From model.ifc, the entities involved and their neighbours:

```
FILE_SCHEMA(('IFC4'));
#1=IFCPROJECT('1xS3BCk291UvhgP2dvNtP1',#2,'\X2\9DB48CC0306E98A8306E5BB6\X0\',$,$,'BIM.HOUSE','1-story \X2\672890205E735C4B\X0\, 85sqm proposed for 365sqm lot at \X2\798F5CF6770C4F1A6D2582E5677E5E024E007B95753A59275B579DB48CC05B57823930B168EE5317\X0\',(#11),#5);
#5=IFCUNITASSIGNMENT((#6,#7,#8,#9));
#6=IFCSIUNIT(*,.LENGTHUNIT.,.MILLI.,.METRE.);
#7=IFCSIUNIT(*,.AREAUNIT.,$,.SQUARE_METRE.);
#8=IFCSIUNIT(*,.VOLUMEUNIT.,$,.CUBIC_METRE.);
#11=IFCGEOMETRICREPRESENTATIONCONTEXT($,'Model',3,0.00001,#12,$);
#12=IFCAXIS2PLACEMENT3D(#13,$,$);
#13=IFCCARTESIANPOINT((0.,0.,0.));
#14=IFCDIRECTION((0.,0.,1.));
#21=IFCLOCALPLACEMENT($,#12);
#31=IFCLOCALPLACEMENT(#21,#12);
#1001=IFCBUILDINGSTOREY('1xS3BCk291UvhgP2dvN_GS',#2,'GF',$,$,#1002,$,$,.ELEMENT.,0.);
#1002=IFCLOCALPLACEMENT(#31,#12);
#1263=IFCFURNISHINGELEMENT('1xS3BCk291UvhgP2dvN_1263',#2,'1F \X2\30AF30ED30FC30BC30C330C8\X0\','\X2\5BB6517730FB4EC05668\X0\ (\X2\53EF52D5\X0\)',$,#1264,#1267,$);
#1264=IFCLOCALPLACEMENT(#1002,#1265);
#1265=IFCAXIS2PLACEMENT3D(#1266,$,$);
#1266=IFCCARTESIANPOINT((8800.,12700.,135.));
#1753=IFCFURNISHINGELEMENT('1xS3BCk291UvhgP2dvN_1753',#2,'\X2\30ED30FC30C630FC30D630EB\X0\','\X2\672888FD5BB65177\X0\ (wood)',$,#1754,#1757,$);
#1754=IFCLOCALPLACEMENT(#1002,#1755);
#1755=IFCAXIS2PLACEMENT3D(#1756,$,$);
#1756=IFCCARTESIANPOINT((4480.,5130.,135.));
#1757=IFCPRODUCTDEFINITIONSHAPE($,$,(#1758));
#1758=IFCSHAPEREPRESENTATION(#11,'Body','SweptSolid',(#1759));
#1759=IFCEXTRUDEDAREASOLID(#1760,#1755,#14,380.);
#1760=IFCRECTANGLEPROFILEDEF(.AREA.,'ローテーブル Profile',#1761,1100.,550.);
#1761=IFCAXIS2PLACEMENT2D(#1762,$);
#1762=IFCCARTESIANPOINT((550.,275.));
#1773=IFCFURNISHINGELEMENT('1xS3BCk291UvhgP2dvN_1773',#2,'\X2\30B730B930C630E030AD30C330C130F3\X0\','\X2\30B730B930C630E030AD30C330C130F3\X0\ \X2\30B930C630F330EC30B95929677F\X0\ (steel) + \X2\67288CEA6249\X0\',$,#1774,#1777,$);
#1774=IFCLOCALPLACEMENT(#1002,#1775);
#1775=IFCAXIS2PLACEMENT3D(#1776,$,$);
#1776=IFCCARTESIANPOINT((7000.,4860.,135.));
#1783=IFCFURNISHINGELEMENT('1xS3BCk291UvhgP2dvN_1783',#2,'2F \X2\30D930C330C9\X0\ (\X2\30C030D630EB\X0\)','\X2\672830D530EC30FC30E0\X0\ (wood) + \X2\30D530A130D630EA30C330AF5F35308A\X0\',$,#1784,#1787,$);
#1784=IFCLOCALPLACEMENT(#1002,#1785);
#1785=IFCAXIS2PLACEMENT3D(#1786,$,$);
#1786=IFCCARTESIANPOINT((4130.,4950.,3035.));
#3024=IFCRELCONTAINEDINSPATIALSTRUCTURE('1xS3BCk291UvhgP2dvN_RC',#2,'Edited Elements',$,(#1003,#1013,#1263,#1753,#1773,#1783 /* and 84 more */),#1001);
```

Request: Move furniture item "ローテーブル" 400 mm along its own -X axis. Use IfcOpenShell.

```python
import ifcopenshell
import ifcopenshell.api.geometry
import ifcopenshell.util.placement
import ifcopenshell.util.unit

model = ifcopenshell.open("model.ifc")
unit_scale = ifcopenshell.util.unit.calculate_unit_scale(model)

item = model.by_guid("1xS3BCk291UvhgP2dvN_1753")
matrix = ifcopenshell.util.placement.get_local_placement(item.ObjectPlacement)
matrix[:3, 3] -= matrix[:3, 0] * 0.4 / unit_scale
ifcopenshell.api.geometry.edit_object_placement(model, product=item, matrix=matrix, is_si=False)

print(ifcopenshell.util.placement.get_local_placement(item.ObjectPlacement).round(3) + 0.0)

model.write("model_updated.ifc")
```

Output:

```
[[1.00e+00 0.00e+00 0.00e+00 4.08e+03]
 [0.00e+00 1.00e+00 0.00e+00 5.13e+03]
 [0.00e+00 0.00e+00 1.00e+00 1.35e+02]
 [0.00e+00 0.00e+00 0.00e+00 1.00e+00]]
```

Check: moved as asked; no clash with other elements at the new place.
